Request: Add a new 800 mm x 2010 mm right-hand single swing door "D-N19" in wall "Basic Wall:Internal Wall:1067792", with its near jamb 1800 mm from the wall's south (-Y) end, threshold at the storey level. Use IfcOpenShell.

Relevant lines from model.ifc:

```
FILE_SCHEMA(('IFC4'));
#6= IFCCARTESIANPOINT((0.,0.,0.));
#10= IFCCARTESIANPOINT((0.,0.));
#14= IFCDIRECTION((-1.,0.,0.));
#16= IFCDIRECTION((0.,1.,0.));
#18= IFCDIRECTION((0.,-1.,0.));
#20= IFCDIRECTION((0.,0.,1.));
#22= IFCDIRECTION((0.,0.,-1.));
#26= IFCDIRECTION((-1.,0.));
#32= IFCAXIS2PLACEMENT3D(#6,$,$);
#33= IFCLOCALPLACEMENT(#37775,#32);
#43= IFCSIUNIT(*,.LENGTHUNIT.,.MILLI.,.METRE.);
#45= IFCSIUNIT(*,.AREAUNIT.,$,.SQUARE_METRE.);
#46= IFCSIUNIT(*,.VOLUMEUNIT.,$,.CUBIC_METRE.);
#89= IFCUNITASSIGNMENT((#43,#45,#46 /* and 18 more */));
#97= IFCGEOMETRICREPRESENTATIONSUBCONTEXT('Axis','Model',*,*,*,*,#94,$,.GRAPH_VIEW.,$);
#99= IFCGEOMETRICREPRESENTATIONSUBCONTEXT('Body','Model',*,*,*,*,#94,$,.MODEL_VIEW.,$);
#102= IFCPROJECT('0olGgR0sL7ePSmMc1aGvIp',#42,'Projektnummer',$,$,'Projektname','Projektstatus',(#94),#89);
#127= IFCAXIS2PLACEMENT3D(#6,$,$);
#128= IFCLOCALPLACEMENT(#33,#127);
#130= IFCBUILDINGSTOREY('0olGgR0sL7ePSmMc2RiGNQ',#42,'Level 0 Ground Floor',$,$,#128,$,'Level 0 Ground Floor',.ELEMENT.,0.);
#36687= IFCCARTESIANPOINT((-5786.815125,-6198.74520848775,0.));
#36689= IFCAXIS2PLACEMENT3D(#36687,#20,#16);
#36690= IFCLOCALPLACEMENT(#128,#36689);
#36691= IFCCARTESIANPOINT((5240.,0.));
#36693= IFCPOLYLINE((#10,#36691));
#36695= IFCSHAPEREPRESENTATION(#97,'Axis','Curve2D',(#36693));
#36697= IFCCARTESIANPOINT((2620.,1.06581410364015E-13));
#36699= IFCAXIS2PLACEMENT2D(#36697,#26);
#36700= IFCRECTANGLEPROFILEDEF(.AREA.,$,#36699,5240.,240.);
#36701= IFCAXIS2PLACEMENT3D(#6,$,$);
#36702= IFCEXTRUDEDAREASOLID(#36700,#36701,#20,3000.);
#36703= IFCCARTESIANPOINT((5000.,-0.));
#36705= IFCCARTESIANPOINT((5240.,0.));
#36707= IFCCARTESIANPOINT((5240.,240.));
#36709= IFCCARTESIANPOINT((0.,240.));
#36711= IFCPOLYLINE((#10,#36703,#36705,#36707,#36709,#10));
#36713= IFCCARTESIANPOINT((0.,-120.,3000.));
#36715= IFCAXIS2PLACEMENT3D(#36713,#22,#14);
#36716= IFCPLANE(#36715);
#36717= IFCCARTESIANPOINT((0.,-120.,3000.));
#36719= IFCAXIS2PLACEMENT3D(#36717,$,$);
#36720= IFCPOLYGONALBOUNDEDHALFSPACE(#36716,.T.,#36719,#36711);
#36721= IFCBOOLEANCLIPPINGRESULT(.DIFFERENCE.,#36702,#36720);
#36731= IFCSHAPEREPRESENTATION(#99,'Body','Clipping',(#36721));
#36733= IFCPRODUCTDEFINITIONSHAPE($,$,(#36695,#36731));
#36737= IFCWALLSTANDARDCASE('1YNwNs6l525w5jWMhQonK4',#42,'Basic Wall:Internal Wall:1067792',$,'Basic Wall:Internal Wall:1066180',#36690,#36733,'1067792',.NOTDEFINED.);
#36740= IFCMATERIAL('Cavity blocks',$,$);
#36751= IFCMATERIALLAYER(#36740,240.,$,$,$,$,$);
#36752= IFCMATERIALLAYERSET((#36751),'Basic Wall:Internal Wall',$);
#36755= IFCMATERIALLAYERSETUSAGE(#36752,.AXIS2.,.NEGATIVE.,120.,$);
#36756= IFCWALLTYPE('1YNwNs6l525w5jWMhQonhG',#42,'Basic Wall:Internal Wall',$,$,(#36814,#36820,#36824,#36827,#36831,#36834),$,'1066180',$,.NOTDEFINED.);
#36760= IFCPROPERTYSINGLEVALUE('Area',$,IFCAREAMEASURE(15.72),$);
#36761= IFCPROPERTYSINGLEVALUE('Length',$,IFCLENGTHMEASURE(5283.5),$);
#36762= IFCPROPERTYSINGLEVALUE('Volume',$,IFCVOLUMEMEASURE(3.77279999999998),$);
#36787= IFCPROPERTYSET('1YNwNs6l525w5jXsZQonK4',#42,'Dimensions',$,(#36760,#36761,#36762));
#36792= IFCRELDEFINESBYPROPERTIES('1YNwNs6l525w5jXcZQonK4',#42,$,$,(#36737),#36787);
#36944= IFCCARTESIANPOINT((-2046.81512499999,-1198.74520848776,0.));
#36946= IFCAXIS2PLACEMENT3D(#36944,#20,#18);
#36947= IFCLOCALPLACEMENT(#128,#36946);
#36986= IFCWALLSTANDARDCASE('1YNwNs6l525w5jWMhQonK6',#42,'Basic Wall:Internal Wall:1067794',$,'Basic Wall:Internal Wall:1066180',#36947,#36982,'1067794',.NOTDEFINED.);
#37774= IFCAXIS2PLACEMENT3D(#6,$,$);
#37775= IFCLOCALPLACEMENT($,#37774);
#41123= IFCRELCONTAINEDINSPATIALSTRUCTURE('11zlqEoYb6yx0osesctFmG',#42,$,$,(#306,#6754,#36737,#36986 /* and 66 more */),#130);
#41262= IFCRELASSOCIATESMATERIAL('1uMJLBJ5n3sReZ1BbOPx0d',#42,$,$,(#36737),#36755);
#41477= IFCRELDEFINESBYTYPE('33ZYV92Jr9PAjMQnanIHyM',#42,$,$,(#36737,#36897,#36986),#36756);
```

```python
import numpy as np
import ifcopenshell
import ifcopenshell.api.feature
import ifcopenshell.api.geometry
import ifcopenshell.api.pset
import ifcopenshell.api.root
import ifcopenshell.api.spatial
import ifcopenshell.geom
import ifcopenshell.util.element
import ifcopenshell.util.placement
import ifcopenshell.util.representation
import ifcopenshell.util.shape
import ifcopenshell.util.unit

model = ifcopenshell.open("model.ifc")
unit_scale = ifcopenshell.util.unit.calculate_unit_scale(model)
area_scale = ifcopenshell.util.unit.calculate_unit_scale(model, "AREAUNIT")
volume_scale = ifcopenshell.util.unit.calculate_unit_scale(model, "VOLUMEUNIT")
settings = ifcopenshell.geom.settings()


def volume(element):
    """Net volume in cubic metres, openings subtracted."""
    shape = ifcopenshell.geom.create_shape(settings, element)
    return ifcopenshell.util.shape.get_volume(shape.geometry)


wall = model.by_guid("1YNwNs6l525w5jWMhQonK4")
storey = ifcopenshell.util.element.get_container(wall, ifc_class="IfcBuildingStorey")
context = ifcopenshell.util.representation.get_context(model, "Model", "Body", "MODEL_VIEW")
before = volume(wall)

width, height, from_end, sill = 0.8, 2.01, 1.8, 0.0  # metres

# The wall runs along its own X axis, and the end named is its -X end.
wall_shape = ifcopenshell.geom.create_shape(settings, wall)
x, y, z = ifcopenshell.util.shape.get_vertices(wall_shape.geometry).T
start = x.min() + from_end
face, thickness = float(y.min()), float(y.max() - y.min())
wall_matrix = ifcopenshell.util.placement.get_local_placement(wall.ObjectPlacement)
level = ifcopenshell.util.placement.get_local_placement(storey.ObjectPlacement)[2, 3]


def in_wall(x, y):
    """Placement at x, y metres in the wall's axes, at sill height."""
    matrix = wall_matrix.copy()
    matrix[:, 3] = wall_matrix @ np.array([x / unit_scale, y / unit_scale, 0.0, 1.0])
    matrix[2, 3] = level + sill / unit_scale
    return matrix


# Opening: a box that overshoots both wall faces by 50 mm.
opening = ifcopenshell.api.root.create_entity(model, ifc_class="IfcOpeningElement", predefined_type="OPENING")
box = ifcopenshell.api.geometry.add_wall_representation(
    model, context=context, length=width, height=height, thickness=thickness + 0.1
)
ifcopenshell.api.geometry.assign_representation(model, product=opening, representation=box)
ifcopenshell.api.geometry.edit_object_placement(model, product=opening, matrix=in_wall(start, face - 0.05), is_si=False)
ifcopenshell.api.feature.add_feature(model, feature=opening, element=wall)

door = ifcopenshell.api.root.create_entity(model, ifc_class="IfcDoor", name="D-N19", predefined_type="DOOR")
door.OverallWidth, door.OverallHeight = width / unit_scale, height / unit_scale
door.OperationType = "SINGLE_SWING_RIGHT"
body = ifcopenshell.api.geometry.add_door_representation(
    model,
    context=context,
    overall_width=door.OverallWidth,
    overall_height=door.OverallHeight,
    operation_type="SINGLE_SWING_RIGHT",
    lining_properties={"LiningDepth": thickness / unit_scale, "ThresholdDepth": thickness / unit_scale},
)
ifcopenshell.api.geometry.assign_representation(model, product=door, representation=body)
ifcopenshell.api.spatial.assign_container(model, products=[door], relating_structure=storey)
ifcopenshell.api.feature.add_filling(model, opening=opening, element=door)

# The lining spans the wall, so the door starts at the wall face.
ifcopenshell.api.geometry.edit_object_placement(model, product=door, matrix=in_wall(start, face), is_si=False)

after = volume(wall)

# Update the wall's stored quantities.
pset = model.by_id(ifcopenshell.util.element.get_pset(wall, "Dimensions", should_inherit=False)["id"])
ifcopenshell.api.pset.edit_pset(model, pset=pset, properties={
    "Area": model.create_entity("IfcAreaMeasure", after / thickness / area_scale),
    "Volume": model.create_entity("IfcVolumeMeasure", after / volume_scale),
})

print(f"wall volume {before:.3f} -> {after:.3f} m3")

model.write("model_v2.ifc")
```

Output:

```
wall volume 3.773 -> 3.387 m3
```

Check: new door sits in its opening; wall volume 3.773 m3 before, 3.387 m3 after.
